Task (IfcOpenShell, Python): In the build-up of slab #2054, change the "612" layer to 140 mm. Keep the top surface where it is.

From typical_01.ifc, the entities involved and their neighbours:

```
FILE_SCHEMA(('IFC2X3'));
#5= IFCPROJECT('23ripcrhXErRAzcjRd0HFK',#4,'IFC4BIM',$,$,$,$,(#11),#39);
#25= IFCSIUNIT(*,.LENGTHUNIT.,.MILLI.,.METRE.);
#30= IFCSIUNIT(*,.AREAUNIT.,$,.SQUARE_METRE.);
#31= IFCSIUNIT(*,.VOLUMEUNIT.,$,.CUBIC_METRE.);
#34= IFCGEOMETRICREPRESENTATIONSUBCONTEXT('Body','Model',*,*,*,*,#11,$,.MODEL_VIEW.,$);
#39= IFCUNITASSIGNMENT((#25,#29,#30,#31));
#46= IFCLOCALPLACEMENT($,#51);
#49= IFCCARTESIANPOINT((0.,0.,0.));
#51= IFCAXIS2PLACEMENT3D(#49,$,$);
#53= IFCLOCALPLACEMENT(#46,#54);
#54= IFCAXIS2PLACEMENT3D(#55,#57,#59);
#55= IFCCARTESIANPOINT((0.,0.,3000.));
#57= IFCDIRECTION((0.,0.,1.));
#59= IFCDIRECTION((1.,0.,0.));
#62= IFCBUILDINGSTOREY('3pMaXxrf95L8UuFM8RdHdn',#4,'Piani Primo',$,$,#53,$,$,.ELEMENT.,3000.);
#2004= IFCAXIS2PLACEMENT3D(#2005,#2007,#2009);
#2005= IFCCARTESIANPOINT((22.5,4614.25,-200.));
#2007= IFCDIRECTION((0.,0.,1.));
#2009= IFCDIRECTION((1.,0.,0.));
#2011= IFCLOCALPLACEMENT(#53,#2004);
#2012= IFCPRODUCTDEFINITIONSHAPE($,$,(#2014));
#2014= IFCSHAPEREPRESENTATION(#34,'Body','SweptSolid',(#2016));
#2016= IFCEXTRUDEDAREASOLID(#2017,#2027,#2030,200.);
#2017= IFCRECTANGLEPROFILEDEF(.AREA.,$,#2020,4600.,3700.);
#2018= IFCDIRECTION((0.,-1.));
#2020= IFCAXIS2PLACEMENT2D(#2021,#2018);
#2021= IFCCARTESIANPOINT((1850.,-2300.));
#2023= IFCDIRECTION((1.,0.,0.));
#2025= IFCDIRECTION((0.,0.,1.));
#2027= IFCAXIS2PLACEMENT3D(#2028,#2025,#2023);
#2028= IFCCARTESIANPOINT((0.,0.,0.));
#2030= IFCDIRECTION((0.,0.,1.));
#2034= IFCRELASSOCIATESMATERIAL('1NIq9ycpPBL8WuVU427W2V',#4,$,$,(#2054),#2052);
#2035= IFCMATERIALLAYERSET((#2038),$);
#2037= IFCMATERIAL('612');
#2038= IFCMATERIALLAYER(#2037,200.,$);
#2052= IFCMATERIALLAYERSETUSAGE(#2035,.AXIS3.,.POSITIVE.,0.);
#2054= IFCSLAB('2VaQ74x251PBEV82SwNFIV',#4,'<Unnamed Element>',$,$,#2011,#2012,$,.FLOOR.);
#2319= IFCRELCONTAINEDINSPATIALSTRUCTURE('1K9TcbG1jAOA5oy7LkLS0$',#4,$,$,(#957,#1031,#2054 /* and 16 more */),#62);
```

```python
import ifcopenshell
import ifcopenshell.util.element
import ifcopenshell.util.representation
import ifcopenshell.util.unit

model = ifcopenshell.open("typical_01.ifc")
unit_scale = ifcopenshell.util.unit.calculate_unit_scale(model)

layer_set = model.by_id(2035)
layer = next(l for l in layer_set.MaterialLayers if l.Material and l.Material.Name == "612")
change = 0.14 / unit_scale - layer.LayerThickness
layer.LayerThickness += change

# Geometry does not follow the layer set by itself.
slabs = [e for e in ifcopenshell.util.element.get_elements_by_material(model, layer_set) if e.is_a("IfcSlab")]
for slab in sorted(slabs, key=lambda e: e.id()):
    body = ifcopenshell.util.representation.get_representation(slab, "Model", "Body")
    solid = body.Items[0]
    old_depth = solid.Depth
    solid.Depth += change
    # Extruded upwards: lower the start of the extrusion so the top stays.
    x, y, z = solid.Position.Location.Coordinates
    solid.Position.Location = model.createIfcCartesianPoint((x, y, z - change))
    print(slab.id(), f"{old_depth:g} -> {solid.Depth:g}")

# The layers are counted up from the underside, which has moved.
for usage in {ifcopenshell.util.element.get_material(slab) for slab in slabs}:
    usage.OffsetFromReferenceLine -= change

model.write("typical_01_rev.ifc")
```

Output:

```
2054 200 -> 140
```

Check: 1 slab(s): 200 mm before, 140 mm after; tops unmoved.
